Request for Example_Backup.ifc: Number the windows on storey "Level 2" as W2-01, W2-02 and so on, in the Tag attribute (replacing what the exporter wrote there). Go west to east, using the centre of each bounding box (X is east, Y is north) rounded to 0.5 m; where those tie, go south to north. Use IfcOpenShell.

First a look at what the model holds.

```python
import ifcopenshell
import ifcopenshell.util.element
import ifcopenshell.util.placement

model = ifcopenshell.open("Example_Backup.ifc")
print(model.schema)
storey = next(s for s in model.by_type("IfcBuildingStorey") if s.Name == "Level 2")
windows = [e for e in ifcopenshell.util.element.get_decomposition(storey) if e.is_a("IfcWindow")]
for e in sorted(windows, key=lambda e: e.id()):
    origin = ifcopenshell.util.placement.get_local_placement(e.ObjectPlacement)[:3, 3]
    print(e.id(), e.Tag, e.Name, origin.round(2) + 0.0, sep=" | ")
```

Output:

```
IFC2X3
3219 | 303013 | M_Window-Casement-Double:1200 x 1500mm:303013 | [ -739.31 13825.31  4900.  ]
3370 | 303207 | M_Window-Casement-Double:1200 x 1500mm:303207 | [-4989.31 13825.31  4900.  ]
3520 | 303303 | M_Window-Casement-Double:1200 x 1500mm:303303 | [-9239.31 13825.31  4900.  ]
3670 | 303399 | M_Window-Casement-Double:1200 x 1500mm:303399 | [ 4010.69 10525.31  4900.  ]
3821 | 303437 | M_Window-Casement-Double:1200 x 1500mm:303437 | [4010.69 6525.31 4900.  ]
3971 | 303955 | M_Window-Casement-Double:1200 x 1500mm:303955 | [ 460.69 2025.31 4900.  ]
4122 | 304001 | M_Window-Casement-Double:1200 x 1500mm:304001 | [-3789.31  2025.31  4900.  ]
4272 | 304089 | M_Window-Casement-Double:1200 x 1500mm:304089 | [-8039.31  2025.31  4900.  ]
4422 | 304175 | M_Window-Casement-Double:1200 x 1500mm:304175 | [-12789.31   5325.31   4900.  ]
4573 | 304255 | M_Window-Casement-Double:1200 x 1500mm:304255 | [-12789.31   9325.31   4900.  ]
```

```python
import ifcopenshell
import ifcopenshell.geom
import ifcopenshell.util.element
import ifcopenshell.util.shape

model = ifcopenshell.open("Example_Backup.ifc")
settings = ifcopenshell.geom.settings()
settings.set("use-world-coords", True)


def centre(element):
    shape = ifcopenshell.geom.create_shape(settings, element)
    return ifcopenshell.util.shape.get_bbox_centroid(shape.geometry)


storey = next(s for s in model.by_type("IfcBuildingStorey") if s.Name == "Level 2")
windows = [e for e in ifcopenshell.util.element.get_decomposition(storey) if e.is_a("IfcWindow")]

# Insertion points can sit at a corner or the storey origin, so sort by the geometry (in metres).
centres = {e: centre(e) for e in windows}
windows.sort(key=lambda e: (round(centres[e][0] / 0.5), centres[e][1]))

for i, e in enumerate(windows, start=1):
    number = f"W2-{i:02d}"
    e.Tag = number
    print(e.id(), number)

model.write("Example_Backup_edited.ifc")
```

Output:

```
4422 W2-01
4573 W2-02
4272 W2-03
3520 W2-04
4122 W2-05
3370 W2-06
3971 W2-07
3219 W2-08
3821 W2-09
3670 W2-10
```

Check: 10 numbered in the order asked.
